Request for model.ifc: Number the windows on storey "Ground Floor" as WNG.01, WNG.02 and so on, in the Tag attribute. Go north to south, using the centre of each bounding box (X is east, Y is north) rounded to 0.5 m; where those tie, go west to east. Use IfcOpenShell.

First a look at what the model holds.

```python
import ifcopenshell
import ifcopenshell.util.element
import ifcopenshell.util.placement

model = ifcopenshell.open("model.ifc")
print(model.schema)
storey = next(s for s in model.by_type("IfcBuildingStorey") if s.Name == "Ground Floor")
windows = [e for e in ifcopenshell.util.element.get_decomposition(storey) if e.is_a("IfcWindow")]
for e in sorted(windows, key=lambda e: e.id()):
    origin = ifcopenshell.util.placement.get_local_placement(e.ObjectPlacement)[:3, 3]
    print(e.id(), e.Tag, e.Name, origin.round(2) + 0.0, sep=" | ")
```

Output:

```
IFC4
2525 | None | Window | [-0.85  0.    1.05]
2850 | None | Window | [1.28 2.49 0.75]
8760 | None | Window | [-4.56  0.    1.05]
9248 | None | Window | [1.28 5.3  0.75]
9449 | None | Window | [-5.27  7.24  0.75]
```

```python
import ifcopenshell
import ifcopenshell.geom
import ifcopenshell.util.element
import ifcopenshell.util.shape

model = ifcopenshell.open("model.ifc")
settings = ifcopenshell.geom.settings()
settings.set("use-world-coords", True)


def centre(element):
    shape = ifcopenshell.geom.create_shape(settings, element)
    return ifcopenshell.util.shape.get_bbox_centroid(shape.geometry)


storey = next(s for s in model.by_type("IfcBuildingStorey") if s.Name == "Ground Floor")
windows = [e for e in ifcopenshell.util.element.get_decomposition(storey) if e.is_a("IfcWindow")]

# Insertion points can sit at a corner or the storey origin, so sort by the geometry (in metres).
centres = {e: centre(e) for e in windows}
windows.sort(key=lambda e: (-round(centres[e][1] / 0.5), centres[e][0]))

for i, e in enumerate(windows, start=1):
    number = f"WNG.{i:02d}"
    e.Tag = number
    print(e.id(), number)

model.write("model_rev.ifc")
```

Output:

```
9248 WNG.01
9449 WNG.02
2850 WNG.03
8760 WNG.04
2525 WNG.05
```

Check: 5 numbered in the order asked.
